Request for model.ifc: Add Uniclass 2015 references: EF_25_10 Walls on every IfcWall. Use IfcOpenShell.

First a look at what the model holds.

```python
import ifcopenshell

model = ifcopenshell.open("model.ifc")
print(model.schema)
print("classifications:", [c.Name for c in model.by_type("IfcClassification")])
for ifc_class in ("IfcDoor", "IfcRoof", "IfcStair", "IfcWall", "IfcWindow"):
    print(ifc_class, len(model.by_type(ifc_class)))
```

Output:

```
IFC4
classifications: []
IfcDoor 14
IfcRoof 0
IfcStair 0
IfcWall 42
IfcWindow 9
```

```python
import ifcopenshell
import ifcopenshell.api.classification

model = ifcopenshell.open("model.ifc")

system = ifcopenshell.api.classification.add_classification(model, classification="Uniclass 2015")

codes = {
    "IfcWall": ("EF_25_10", "Walls"),
}
for ifc_class, (code, name) in codes.items():
    products = model.by_type(ifc_class)
    ifcopenshell.api.classification.add_reference(
        model, products=products, classification=system, identification=code, name=name
    )
    print(code, len(products))

model.write("model_edited.ifc")
```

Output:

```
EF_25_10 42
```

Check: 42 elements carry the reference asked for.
